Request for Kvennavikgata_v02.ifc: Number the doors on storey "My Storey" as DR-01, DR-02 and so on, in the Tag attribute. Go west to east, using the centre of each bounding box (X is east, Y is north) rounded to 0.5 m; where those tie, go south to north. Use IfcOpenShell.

First a look at what the model holds.

```python
import ifcopenshell
import ifcopenshell.util.element
import ifcopenshell.util.placement

model = ifcopenshell.open("Kvennavikgata_v02.ifc")
print(model.schema)
storey = next(s for s in model.by_type("IfcBuildingStorey") if s.Name == "My Storey")
doors = [e for e in ifcopenshell.util.element.get_decomposition(storey) if e.is_a("IfcDoor")]
for e in sorted(doors, key=lambda e: e.id()):
    origin = ifcopenshell.util.placement.get_local_placement(e.ObjectPlacement)[:3, 3]
    print(e.id(), e.Tag, e.Name, origin.round(2) + 0.0, sep=" | ")
```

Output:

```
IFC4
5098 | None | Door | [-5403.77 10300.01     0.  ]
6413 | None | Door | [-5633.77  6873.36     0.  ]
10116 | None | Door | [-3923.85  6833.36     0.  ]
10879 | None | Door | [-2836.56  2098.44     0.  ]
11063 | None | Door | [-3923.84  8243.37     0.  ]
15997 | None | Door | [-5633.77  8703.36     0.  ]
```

```python
import ifcopenshell
import ifcopenshell.geom
import ifcopenshell.util.element
import ifcopenshell.util.shape

model = ifcopenshell.open("Kvennavikgata_v02.ifc")
settings = ifcopenshell.geom.settings()
settings.set("use-world-coords", True)


def centre(element):
    shape = ifcopenshell.geom.create_shape(settings, element)
    return ifcopenshell.util.shape.get_bbox_centroid(shape.geometry)


storey = next(s for s in model.by_type("IfcBuildingStorey") if s.Name == "My Storey")
doors = [e for e in ifcopenshell.util.element.get_decomposition(storey) if e.is_a("IfcDoor")]

# Insertion points can sit at a corner or the storey origin, so sort by the geometry (in metres).
centres = {e: centre(e) for e in doors}
doors.sort(key=lambda e: (round(centres[e][0] / 0.5), centres[e][1]))

for i, e in enumerate(doors, start=1):
    number = f"DR-{i:02d}"
    e.Tag = number
    print(e.id(), number)

model.write("Kvennavikgata_v02_rev.ifc")
```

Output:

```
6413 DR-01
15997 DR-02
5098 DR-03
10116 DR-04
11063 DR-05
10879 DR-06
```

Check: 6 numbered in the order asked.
